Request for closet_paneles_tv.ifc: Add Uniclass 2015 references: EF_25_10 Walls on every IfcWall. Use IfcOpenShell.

First a look at what the model holds.

```python
import ifcopenshell

model = ifcopenshell.open("closet_paneles_tv.ifc")
print(model.schema)
print("classifications:", [c.Name for c in model.by_type("IfcClassification")])
for ifc_class in ("IfcDoor", "IfcRoof", "IfcStair", "IfcWall", "IfcWindow"):
    print(ifc_class, len(model.by_type(ifc_class)))
```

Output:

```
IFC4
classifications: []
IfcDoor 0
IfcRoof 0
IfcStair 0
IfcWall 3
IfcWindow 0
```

```python
import ifcopenshell
import ifcopenshell.api.classification

model = ifcopenshell.open("closet_paneles_tv.ifc")

system = ifcopenshell.api.classification.add_classification(model, classification="Uniclass 2015")

codes = {
    "IfcWall": ("EF_25_10", "Walls"),
}
for ifc_class, (code, name) in codes.items():
    products = model.by_type(ifc_class)
    ifcopenshell.api.classification.add_reference(
        model, products=products, classification=system, identification=code, name=name
    )
    print(code, len(products))

model.write("closet_paneles_tv_updated.ifc")
```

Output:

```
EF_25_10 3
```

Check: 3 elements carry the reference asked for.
